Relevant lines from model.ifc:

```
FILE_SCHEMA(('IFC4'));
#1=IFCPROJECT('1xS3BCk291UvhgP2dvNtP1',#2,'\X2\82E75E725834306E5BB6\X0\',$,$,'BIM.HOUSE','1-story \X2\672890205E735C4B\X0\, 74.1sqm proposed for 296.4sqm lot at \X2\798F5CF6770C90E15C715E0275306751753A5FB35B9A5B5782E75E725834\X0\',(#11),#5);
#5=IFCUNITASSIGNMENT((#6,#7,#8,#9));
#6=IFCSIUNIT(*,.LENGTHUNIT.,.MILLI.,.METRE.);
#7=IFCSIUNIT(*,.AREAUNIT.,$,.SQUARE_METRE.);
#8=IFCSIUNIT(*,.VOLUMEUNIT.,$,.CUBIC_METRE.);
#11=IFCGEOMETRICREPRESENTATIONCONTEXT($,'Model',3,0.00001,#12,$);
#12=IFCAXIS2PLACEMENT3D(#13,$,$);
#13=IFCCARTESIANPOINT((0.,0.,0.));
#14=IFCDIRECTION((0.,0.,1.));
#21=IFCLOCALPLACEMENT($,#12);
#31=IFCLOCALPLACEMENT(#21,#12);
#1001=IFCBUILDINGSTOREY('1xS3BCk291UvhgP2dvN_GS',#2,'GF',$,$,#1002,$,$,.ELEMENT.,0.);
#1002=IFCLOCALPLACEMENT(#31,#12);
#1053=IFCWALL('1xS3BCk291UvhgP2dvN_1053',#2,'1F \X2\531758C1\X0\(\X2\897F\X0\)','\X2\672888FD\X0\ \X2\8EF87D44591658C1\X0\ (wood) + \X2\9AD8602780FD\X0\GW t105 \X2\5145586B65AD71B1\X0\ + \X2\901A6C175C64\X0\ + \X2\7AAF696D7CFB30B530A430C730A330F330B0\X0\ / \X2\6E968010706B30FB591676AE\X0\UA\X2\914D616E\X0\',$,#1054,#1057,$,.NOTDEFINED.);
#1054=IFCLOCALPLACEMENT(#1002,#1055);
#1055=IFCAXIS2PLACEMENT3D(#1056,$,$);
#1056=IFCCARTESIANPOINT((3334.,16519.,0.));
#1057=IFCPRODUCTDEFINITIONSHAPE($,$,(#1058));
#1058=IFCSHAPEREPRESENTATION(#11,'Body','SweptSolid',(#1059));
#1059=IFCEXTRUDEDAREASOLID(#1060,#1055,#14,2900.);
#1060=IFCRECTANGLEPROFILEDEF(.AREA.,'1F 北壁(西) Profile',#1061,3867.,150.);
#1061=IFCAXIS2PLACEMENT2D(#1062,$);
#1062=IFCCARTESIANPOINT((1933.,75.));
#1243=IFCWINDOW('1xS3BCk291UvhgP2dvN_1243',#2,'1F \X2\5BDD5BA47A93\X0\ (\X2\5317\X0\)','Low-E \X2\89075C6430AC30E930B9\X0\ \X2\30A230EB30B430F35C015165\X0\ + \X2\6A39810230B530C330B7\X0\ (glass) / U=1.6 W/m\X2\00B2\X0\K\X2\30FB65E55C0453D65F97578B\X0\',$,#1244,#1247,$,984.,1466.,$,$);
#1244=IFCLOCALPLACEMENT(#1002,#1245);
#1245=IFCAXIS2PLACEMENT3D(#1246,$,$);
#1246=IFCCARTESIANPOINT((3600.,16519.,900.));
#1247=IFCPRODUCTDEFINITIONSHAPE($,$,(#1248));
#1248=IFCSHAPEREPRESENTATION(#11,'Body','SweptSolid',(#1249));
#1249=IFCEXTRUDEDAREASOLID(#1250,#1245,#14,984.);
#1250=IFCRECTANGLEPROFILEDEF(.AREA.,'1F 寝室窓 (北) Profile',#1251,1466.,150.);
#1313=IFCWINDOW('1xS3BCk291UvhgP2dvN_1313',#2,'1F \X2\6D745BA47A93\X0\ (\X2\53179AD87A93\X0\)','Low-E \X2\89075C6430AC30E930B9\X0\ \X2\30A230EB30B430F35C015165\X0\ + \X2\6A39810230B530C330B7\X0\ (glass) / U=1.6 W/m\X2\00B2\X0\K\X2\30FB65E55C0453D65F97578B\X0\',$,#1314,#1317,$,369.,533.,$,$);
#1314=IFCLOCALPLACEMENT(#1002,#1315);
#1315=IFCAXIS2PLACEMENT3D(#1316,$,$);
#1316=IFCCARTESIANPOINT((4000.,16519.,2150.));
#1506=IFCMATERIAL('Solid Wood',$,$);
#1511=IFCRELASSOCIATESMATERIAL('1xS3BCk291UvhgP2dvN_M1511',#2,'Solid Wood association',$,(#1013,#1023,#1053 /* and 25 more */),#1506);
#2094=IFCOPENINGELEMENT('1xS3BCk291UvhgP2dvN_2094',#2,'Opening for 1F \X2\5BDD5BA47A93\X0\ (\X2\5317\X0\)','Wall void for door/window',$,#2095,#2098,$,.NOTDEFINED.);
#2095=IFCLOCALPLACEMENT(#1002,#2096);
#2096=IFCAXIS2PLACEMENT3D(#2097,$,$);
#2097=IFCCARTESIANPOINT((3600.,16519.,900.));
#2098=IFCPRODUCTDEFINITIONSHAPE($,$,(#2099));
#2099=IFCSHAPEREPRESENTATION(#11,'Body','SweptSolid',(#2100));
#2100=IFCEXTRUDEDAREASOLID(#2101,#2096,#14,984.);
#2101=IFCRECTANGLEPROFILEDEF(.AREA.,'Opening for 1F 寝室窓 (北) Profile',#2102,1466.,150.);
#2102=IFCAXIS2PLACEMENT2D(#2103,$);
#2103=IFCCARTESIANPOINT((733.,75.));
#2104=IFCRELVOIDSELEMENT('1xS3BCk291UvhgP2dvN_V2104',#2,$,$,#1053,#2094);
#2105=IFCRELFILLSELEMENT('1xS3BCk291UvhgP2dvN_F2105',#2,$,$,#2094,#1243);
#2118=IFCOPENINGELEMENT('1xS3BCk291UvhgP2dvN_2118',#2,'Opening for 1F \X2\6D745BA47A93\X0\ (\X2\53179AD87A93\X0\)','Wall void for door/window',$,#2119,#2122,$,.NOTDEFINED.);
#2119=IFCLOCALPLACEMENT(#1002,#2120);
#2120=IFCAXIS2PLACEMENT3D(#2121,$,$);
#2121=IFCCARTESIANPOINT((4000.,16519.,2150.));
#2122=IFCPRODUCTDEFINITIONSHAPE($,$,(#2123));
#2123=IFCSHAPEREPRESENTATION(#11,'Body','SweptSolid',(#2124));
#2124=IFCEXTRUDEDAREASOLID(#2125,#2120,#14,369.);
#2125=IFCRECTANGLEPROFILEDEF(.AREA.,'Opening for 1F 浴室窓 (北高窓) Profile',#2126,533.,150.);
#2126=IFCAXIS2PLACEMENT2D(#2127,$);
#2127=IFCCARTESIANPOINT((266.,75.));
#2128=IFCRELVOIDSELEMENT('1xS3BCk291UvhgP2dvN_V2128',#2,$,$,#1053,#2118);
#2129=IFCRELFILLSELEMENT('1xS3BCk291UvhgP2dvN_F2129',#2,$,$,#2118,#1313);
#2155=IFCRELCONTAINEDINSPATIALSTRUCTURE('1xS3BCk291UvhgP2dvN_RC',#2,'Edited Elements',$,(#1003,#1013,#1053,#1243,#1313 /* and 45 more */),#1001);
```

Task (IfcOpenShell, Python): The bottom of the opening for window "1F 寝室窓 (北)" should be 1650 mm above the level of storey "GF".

```python
import numpy as np
import ifcopenshell
import ifcopenshell.api.geometry
import ifcopenshell.geom
import ifcopenshell.util.element
import ifcopenshell.util.placement
import ifcopenshell.util.shape
import ifcopenshell.util.unit

model = ifcopenshell.open("model.ifc")
unit_scale = ifcopenshell.util.unit.calculate_unit_scale(model)

window = model.by_guid("1xS3BCk291UvhgP2dvN_1243")
opening = window.FillsVoids[0].RelatingOpeningElement
storey = ifcopenshell.util.element.get_container(window, ifc_class="IfcBuildingStorey")
level = ifcopenshell.util.placement.get_local_placement(storey.ObjectPlacement)[2, 3]

# The opening's origin need not be at the sill, so measure its lowest point.
shape = ifcopenshell.geom.create_shape(ifcopenshell.geom.settings(), opening)
bottom = ifcopenshell.util.shape.get_shape_bottom_elevation(shape, shape.geometry) / unit_scale
dz = level + 1.65 / unit_scale - bottom

shift = np.array([0.0, 0.0, dz])
# The window is not placed relative to its opening, so move both.
for product in (opening, window):
    matrix = ifcopenshell.util.placement.get_local_placement(product.ObjectPlacement)
    matrix[:3, 3] += shift
    ifcopenshell.api.geometry.edit_object_placement(model, product=product, matrix=matrix, is_si=False)

print(f"moved by {dz * unit_scale:+.3f} m")

model.write("model_v2.ifc")
```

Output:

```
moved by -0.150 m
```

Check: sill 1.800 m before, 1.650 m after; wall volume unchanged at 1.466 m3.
